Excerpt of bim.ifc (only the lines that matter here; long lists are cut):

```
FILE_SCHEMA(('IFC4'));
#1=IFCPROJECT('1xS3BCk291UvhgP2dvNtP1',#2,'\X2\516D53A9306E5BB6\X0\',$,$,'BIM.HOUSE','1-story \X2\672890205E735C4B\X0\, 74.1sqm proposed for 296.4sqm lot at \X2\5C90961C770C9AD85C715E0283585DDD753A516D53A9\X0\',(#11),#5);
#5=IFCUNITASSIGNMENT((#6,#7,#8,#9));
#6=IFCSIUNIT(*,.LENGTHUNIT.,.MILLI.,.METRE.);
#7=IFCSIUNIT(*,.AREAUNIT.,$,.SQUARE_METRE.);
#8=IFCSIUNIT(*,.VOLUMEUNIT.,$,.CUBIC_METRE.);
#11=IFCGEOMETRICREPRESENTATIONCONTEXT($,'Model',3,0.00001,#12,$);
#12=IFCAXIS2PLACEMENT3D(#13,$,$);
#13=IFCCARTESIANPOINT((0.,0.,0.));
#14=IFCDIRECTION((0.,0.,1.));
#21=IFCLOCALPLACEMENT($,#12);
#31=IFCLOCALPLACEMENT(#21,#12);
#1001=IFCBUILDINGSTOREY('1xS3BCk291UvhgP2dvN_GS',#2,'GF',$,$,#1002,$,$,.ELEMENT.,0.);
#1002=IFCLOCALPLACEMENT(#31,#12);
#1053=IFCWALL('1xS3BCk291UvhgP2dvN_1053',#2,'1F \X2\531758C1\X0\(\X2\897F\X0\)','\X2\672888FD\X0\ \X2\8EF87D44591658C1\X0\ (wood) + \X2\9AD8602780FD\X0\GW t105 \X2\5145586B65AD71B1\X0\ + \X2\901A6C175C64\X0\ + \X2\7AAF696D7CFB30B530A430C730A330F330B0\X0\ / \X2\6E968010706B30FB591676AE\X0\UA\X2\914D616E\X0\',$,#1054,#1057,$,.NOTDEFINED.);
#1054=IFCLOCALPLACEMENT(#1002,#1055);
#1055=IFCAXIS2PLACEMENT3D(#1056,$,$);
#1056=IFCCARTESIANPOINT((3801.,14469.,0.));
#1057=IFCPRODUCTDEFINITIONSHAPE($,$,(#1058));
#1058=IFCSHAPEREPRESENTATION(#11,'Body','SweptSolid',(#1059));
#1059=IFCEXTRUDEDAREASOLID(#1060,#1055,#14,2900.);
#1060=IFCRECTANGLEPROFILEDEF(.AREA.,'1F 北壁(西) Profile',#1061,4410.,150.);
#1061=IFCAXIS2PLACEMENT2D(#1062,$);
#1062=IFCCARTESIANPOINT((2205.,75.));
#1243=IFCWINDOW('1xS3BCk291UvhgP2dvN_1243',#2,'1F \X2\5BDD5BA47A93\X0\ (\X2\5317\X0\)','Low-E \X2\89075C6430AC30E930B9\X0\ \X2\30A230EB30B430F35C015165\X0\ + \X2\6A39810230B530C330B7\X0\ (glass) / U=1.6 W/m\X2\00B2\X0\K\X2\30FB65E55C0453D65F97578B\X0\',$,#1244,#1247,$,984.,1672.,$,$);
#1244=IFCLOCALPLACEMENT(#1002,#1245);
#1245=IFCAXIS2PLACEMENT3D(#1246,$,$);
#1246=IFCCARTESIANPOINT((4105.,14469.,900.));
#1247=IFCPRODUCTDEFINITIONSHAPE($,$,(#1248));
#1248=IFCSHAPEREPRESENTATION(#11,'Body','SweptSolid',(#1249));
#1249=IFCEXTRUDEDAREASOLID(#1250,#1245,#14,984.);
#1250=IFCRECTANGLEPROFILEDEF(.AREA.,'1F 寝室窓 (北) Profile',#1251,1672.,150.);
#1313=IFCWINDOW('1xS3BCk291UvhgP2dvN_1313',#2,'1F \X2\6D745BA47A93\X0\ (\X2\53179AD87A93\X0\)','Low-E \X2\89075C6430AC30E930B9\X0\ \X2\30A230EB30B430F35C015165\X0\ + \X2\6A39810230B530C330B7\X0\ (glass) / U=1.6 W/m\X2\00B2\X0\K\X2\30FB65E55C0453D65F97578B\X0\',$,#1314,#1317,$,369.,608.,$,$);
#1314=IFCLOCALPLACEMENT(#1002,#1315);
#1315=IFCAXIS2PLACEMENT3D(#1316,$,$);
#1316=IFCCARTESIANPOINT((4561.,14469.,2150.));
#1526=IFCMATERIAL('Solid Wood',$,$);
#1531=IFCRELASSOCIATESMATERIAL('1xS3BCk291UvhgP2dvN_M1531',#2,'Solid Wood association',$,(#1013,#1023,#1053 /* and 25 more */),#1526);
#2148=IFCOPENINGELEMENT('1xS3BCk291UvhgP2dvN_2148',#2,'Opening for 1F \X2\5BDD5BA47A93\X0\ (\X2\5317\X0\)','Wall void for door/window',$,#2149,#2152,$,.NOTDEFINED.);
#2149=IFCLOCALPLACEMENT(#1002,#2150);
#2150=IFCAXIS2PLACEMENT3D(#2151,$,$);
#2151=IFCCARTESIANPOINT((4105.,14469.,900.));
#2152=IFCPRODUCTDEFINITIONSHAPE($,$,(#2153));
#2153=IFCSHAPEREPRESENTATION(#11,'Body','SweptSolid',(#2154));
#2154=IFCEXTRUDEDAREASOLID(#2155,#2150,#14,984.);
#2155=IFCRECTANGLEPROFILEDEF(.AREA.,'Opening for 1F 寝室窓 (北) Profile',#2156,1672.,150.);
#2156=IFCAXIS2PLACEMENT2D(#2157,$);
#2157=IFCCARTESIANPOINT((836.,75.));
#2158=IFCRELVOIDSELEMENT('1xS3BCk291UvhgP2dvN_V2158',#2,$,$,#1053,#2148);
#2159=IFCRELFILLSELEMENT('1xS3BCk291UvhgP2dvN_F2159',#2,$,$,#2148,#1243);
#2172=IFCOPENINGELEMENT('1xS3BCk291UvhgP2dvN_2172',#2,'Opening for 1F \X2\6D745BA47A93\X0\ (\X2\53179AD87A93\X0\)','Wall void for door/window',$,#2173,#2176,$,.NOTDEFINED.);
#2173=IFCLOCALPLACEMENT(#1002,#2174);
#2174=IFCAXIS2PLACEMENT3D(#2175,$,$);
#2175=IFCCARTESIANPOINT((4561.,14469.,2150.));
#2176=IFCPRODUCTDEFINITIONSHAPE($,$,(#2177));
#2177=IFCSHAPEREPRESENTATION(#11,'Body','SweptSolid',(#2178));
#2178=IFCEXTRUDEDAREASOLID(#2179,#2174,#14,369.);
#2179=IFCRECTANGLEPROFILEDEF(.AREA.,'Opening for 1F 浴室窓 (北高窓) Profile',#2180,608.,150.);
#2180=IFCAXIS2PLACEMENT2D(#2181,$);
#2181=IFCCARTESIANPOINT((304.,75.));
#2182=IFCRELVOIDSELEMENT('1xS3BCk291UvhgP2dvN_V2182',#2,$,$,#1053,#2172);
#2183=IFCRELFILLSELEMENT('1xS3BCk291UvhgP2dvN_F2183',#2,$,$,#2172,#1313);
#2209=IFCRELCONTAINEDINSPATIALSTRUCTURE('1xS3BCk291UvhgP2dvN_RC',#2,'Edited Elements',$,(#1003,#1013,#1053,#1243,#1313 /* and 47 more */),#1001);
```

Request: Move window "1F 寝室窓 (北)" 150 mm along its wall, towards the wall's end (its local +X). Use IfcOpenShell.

```python
import ifcopenshell
import ifcopenshell.api.geometry
import ifcopenshell.util.placement
import ifcopenshell.util.unit

model = ifcopenshell.open("bim.ifc")
unit_scale = ifcopenshell.util.unit.calculate_unit_scale(model)

window = model.by_id(1243)
opening = window.FillsVoids[0].RelatingOpeningElement
wall = opening.VoidsElements[0].RelatingBuildingElement

wall_matrix = ifcopenshell.util.placement.get_local_placement(wall.ObjectPlacement)
shift = wall_matrix[:3, 0] * 0.15 / unit_scale
before = ifcopenshell.util.placement.get_local_placement(window.ObjectPlacement)[:3, 3].copy()

# The window is not placed relative to its opening, so move both.
for product in (opening, window):
    matrix = ifcopenshell.util.placement.get_local_placement(product.ObjectPlacement)
    matrix[:3, 3] += shift
    ifcopenshell.api.geometry.edit_object_placement(model, product=product, matrix=matrix, is_si=False)

after = ifcopenshell.util.placement.get_local_placement(window.ObjectPlacement)[:3, 3]
print("window moved by", (after - before).round(3) + 0.0)

model.write("bim_rev.ifc")
```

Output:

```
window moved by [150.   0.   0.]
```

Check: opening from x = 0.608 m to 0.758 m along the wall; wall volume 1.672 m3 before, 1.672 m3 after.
